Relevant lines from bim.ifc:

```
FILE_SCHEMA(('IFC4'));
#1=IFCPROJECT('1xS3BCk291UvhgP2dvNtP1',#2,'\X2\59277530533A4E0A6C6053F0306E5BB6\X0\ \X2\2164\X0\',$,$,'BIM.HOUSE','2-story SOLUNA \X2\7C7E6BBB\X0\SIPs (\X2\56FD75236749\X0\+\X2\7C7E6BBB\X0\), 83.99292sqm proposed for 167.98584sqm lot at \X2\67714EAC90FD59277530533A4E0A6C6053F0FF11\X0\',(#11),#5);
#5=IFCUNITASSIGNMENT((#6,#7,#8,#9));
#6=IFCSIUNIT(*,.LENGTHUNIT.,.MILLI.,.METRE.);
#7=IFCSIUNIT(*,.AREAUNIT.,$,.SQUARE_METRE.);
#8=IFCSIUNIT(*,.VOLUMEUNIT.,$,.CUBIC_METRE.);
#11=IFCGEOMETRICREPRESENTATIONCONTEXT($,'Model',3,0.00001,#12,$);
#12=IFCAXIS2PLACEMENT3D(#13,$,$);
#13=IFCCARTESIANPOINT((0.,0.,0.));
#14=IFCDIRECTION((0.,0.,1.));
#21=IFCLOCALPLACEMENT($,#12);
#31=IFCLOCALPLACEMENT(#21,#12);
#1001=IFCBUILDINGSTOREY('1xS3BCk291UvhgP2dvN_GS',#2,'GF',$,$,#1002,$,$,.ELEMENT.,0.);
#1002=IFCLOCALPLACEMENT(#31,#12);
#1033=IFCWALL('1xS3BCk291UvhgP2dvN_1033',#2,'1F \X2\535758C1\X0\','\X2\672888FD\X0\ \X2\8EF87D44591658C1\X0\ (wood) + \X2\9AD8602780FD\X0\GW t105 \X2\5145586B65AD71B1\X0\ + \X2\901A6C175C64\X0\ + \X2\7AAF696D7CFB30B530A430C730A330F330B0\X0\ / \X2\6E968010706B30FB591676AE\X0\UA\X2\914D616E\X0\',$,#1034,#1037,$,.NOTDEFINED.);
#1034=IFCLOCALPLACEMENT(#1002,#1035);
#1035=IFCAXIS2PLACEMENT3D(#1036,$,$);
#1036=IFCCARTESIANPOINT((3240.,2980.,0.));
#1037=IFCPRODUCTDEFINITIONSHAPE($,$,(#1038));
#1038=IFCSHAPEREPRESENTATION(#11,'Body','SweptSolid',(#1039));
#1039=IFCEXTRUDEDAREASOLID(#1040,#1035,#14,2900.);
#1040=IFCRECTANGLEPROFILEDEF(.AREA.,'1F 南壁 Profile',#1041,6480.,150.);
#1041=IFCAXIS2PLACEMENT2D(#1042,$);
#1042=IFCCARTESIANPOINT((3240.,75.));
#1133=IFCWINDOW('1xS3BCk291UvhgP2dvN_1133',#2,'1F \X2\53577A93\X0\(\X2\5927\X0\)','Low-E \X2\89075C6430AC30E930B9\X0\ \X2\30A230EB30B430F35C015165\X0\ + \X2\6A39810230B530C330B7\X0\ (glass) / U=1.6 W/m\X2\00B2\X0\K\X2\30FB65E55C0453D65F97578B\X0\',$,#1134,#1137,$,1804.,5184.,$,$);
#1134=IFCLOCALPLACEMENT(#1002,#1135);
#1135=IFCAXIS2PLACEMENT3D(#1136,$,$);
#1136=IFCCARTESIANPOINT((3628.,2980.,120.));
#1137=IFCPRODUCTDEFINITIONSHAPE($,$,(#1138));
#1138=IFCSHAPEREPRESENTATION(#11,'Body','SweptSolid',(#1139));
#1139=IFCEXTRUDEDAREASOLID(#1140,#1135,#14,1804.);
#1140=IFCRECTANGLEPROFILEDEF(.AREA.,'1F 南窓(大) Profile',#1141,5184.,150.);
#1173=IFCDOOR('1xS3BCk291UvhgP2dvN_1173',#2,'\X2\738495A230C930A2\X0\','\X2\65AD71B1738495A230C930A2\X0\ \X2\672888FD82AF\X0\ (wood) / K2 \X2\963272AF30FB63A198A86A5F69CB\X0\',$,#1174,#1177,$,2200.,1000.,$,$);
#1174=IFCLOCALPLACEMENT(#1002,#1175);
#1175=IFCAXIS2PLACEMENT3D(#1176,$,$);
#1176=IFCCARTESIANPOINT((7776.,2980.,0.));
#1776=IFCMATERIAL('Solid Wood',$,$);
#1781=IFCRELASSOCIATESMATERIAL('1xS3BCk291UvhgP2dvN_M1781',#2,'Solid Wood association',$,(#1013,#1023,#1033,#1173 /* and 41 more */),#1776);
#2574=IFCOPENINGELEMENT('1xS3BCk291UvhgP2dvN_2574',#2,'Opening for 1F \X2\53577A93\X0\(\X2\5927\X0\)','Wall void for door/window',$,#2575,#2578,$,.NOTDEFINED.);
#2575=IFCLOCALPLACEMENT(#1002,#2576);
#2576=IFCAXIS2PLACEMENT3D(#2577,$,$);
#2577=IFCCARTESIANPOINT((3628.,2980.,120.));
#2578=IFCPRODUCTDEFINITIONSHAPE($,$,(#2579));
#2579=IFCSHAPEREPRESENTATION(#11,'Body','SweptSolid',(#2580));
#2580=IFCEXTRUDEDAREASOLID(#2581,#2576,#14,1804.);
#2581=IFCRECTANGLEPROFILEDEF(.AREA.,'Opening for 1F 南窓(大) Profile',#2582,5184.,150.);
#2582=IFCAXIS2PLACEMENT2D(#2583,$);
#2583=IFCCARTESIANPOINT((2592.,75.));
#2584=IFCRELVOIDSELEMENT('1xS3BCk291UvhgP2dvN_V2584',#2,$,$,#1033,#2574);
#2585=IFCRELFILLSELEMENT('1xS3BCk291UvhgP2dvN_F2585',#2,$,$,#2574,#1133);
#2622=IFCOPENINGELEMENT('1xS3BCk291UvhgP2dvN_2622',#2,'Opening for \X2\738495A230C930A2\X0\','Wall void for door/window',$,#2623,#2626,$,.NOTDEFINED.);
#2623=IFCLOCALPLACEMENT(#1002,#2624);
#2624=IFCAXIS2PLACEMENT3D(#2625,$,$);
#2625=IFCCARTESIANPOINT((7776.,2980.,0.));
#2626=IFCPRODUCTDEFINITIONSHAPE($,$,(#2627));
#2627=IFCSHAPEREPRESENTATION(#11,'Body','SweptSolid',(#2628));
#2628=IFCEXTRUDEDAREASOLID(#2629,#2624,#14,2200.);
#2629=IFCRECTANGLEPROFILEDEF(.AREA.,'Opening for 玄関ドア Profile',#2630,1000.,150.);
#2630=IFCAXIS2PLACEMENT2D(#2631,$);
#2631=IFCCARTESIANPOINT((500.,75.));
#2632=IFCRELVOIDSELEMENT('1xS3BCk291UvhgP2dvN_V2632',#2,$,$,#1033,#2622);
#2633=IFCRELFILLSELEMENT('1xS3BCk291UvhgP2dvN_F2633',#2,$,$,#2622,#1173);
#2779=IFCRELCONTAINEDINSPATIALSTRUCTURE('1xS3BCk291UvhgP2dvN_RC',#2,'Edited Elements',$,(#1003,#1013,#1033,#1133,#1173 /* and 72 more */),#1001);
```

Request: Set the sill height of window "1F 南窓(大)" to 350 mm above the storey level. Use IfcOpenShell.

```python
import numpy as np
import ifcopenshell
import ifcopenshell.api.geometry
import ifcopenshell.geom
import ifcopenshell.util.element
import ifcopenshell.util.placement
import ifcopenshell.util.shape
import ifcopenshell.util.unit

model = ifcopenshell.open("bim.ifc")
unit_scale = ifcopenshell.util.unit.calculate_unit_scale(model)

window = model.by_id(1133)
opening = window.FillsVoids[0].RelatingOpeningElement
storey = ifcopenshell.util.element.get_container(window, ifc_class="IfcBuildingStorey")
level = ifcopenshell.util.placement.get_local_placement(storey.ObjectPlacement)[2, 3]

# The opening's origin need not be at the sill, so measure its lowest point.
shape = ifcopenshell.geom.create_shape(ifcopenshell.geom.settings(), opening)
bottom = ifcopenshell.util.shape.get_shape_bottom_elevation(shape, shape.geometry) / unit_scale
dz = level + 0.35 / unit_scale - bottom

shift = np.array([0.0, 0.0, dz])
# The window is not placed relative to its opening, so move both.
for product in (opening, window):
    matrix = ifcopenshell.util.placement.get_local_placement(product.ObjectPlacement)
    matrix[:3, 3] += shift
    ifcopenshell.api.geometry.edit_object_placement(model, product=product, matrix=matrix, is_si=False)

print(f"moved by {dz * unit_scale:+.3f} m")

model.write("bim_updated.ifc")
```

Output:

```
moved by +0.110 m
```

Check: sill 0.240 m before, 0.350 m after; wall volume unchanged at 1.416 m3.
